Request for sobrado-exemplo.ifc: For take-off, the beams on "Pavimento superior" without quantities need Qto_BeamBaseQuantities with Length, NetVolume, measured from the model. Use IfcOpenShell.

First a look at what the model holds.

```python
import ifcopenshell
import ifcopenshell.util.element
import ifcopenshell.util.unit

model = ifcopenshell.open("sobrado-exemplo.ifc")
print(model.schema)
for unit_type in ("LENGTHUNIT", "AREAUNIT", "VOLUMEUNIT"):
    print(unit_type, ifcopenshell.util.unit.calculate_unit_scale(model, unit_type))
storey = next(s for s in model.by_type("IfcBuildingStorey") if s.Name == "Pavimento superior")
beams = [e for e in ifcopenshell.util.element.get_decomposition(storey) if e.is_a("IfcBeam")]
for e in sorted(beams, key=lambda e: e.id()):
    print(e.id(), e.is_a(), e.Name, list(ifcopenshell.util.element.get_psets(e, qtos_only=True)), sep=" | ")
```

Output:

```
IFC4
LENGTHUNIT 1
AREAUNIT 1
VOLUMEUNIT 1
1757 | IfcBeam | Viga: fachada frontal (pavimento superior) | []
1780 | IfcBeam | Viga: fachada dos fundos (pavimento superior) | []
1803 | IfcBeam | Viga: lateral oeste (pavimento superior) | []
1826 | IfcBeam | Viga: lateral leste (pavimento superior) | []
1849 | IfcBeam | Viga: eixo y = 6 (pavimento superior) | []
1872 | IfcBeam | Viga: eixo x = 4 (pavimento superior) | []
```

```python
import ifcopenshell
import ifcopenshell.api.pset
import ifcopenshell.geom
import ifcopenshell.util.element
import ifcopenshell.util.shape
import ifcopenshell.util.unit

model = ifcopenshell.open("sobrado-exemplo.ifc")
unit_scale = ifcopenshell.util.unit.calculate_unit_scale(model)
volume_scale = ifcopenshell.util.unit.calculate_unit_scale(model, "VOLUMEUNIT")
settings = ifcopenshell.geom.settings()

storey = next(s for s in model.by_type("IfcBuildingStorey") if s.Name == "Pavimento superior")
beams = [e for e in ifcopenshell.util.element.get_decomposition(storey) if e.is_a("IfcBeam")]

for e in sorted(beams, key=lambda e: e.id()):
    if ifcopenshell.util.element.get_psets(e, qtos_only=True, should_inherit=False):
        continue
    # Geometry comes back in metres, in the element's own axes.
    shape = ifcopenshell.geom.create_shape(settings, e)
    values = {
        "Length": ifcopenshell.util.shape.get_max_xyz(shape.geometry) / unit_scale,
        "NetVolume": ifcopenshell.util.shape.get_volume(shape.geometry) / volume_scale,
    }
    qto = ifcopenshell.api.pset.add_qto(model, product=e, name="Qto_BeamBaseQuantities")
    ifcopenshell.api.pset.edit_qto(model, qto=qto, properties=values)
    print(e.id(), {k: round(v, 3) for k, v in values.items()})

model.write("sobrado-exemplo_edited.ifc")
```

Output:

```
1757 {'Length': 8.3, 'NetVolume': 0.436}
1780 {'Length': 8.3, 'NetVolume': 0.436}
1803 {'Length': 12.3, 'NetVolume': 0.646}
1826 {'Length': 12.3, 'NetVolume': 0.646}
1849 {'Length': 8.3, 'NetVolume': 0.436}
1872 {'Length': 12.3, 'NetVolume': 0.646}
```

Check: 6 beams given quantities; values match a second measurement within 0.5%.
